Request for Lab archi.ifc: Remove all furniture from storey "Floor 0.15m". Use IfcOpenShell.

First a look at what the model holds.

```python
import ifcopenshell
import ifcopenshell.util.element

model = ifcopenshell.open("Lab archi.ifc")
print(model.schema)
storey = next(s for s in model.by_type("IfcBuildingStorey") if s.Name == "Floor 0.15m")
furniture = [e for e in ifcopenshell.util.element.get_decomposition(storey) if e.is_a("IfcFurnishingElement")]
seen = {}
for e in furniture:
    element_type = ifcopenshell.util.element.get_type(e)
    name = element_type.Name if element_type not in (None, e) else None
    seen[name] = seen.get(name, 0) + 1
for name, count in sorted(seen.items(), key=str):
    print(count, "x", name)
```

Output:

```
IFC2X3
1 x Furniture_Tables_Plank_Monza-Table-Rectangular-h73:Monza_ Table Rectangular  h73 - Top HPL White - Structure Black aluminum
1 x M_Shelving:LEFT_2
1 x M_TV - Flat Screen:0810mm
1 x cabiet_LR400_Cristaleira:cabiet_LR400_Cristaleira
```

```python
import ifcopenshell
import ifcopenshell.api.root
import ifcopenshell.util.element

model = ifcopenshell.open("Lab archi.ifc")

storey = next(s for s in model.by_type("IfcBuildingStorey") if s.Name == "Floor 0.15m")
furniture = [e for e in ifcopenshell.util.element.get_decomposition(storey) if e.is_a("IfcFurnishingElement")]

for e in furniture:
    ifcopenshell.api.root.remove_product(model, product=e)
print(len(furniture), "removed")

model.write("Lab archi_rev.ifc")
```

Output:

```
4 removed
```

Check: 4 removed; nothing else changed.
